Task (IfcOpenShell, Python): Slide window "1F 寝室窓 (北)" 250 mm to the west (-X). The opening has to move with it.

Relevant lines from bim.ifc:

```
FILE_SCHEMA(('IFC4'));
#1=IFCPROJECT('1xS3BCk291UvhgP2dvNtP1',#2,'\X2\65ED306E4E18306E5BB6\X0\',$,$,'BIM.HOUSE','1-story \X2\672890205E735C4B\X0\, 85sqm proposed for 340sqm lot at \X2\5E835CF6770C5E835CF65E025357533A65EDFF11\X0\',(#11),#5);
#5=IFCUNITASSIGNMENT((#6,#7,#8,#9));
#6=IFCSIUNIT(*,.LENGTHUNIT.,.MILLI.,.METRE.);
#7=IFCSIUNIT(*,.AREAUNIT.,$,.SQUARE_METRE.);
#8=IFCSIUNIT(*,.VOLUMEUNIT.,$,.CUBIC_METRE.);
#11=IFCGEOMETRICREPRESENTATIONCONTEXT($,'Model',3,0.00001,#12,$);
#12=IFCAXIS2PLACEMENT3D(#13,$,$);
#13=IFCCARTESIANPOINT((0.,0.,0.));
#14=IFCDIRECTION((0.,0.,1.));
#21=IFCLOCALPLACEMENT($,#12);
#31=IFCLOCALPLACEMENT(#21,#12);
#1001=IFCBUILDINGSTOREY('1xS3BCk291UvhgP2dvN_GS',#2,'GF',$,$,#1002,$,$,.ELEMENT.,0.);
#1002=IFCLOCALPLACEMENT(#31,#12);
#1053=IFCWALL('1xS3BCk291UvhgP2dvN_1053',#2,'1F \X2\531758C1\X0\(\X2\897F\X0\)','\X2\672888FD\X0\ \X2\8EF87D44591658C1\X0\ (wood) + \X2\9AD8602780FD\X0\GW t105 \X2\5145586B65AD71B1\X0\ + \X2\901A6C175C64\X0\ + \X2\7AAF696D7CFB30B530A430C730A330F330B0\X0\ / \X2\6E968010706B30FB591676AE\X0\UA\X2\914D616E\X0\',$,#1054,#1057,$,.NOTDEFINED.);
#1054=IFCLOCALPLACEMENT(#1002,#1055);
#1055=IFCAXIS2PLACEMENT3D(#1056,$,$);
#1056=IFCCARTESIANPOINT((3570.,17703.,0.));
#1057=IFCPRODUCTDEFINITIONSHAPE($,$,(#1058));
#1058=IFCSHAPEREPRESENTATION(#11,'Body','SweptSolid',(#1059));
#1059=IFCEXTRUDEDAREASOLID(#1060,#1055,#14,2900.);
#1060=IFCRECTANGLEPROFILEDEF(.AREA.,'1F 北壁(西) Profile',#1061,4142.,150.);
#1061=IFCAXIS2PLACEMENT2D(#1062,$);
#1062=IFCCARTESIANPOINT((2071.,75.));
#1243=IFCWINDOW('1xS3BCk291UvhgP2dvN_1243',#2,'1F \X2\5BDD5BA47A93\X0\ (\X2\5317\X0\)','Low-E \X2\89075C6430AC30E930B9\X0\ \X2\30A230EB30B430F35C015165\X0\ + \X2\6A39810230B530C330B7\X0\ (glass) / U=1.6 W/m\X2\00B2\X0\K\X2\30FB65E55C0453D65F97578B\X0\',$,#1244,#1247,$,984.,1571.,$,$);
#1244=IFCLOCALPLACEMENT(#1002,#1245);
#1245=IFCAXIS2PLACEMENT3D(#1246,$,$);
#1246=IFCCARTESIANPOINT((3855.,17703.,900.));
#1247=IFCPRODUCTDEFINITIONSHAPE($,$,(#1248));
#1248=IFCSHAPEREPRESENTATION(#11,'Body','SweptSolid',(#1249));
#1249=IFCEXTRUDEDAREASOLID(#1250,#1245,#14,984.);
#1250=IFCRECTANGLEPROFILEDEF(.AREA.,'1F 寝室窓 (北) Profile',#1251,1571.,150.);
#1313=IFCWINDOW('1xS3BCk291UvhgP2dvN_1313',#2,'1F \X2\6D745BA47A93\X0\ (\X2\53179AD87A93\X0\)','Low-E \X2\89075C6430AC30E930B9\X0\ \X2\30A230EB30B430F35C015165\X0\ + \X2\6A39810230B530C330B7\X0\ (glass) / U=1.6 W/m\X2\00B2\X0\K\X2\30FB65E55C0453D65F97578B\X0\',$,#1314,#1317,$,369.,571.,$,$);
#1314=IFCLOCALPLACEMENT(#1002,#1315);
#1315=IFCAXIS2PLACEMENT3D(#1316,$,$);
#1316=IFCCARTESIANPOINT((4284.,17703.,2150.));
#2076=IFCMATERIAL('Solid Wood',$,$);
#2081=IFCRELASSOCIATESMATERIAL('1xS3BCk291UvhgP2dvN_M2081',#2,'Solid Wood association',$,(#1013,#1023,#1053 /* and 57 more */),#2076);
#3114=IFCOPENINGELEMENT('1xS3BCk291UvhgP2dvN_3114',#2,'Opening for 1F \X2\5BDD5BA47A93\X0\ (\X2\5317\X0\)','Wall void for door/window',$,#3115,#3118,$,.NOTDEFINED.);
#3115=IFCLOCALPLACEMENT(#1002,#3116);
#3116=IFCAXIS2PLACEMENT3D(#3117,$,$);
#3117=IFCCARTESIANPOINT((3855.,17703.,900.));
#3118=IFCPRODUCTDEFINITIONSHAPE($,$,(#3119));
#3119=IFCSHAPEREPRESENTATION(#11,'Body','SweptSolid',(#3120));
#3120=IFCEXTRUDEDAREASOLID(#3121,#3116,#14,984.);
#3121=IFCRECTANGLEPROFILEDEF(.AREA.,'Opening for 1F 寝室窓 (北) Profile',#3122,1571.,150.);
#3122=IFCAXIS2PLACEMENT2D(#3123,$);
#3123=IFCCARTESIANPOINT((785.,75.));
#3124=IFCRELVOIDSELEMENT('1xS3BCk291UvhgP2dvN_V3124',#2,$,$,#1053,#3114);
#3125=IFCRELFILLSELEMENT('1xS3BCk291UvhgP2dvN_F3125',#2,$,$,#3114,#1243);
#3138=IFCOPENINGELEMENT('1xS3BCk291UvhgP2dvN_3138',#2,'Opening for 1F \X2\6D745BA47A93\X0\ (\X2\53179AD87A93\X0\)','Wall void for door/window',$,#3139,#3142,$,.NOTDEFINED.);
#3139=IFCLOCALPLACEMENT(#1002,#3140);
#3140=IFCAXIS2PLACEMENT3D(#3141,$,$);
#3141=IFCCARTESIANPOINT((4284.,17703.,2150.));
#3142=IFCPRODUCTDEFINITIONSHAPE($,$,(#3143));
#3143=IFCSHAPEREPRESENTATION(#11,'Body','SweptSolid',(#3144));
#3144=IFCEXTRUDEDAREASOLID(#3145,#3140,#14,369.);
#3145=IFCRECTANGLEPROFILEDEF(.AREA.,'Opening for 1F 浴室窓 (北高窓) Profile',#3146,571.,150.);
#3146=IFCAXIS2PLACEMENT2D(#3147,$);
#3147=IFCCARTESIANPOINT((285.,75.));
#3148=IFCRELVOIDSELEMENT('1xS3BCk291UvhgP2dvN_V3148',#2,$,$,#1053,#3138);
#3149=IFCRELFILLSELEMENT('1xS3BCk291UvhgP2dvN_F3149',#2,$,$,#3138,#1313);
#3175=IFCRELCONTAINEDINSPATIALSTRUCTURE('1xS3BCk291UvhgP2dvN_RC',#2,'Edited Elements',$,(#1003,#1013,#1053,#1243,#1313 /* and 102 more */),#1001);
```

```python
import ifcopenshell
import ifcopenshell.api.geometry
import ifcopenshell.util.placement
import ifcopenshell.util.unit

model = ifcopenshell.open("bim.ifc")
unit_scale = ifcopenshell.util.unit.calculate_unit_scale(model)

window = model.by_id(1243)
opening = window.FillsVoids[0].RelatingOpeningElement
wall = opening.VoidsElements[0].RelatingBuildingElement

wall_matrix = ifcopenshell.util.placement.get_local_placement(wall.ObjectPlacement)
shift = wall_matrix[:3, 0] * -0.25 / unit_scale
before = ifcopenshell.util.placement.get_local_placement(window.ObjectPlacement)[:3, 3].copy()

# The window is not placed relative to its opening, so move both.
for product in (opening, window):
    matrix = ifcopenshell.util.placement.get_local_placement(product.ObjectPlacement)
    matrix[:3, 3] += shift
    ifcopenshell.api.geometry.edit_object_placement(model, product=product, matrix=matrix, is_si=False)

after = ifcopenshell.util.placement.get_local_placement(window.ObjectPlacement)[:3, 3]
print("window moved by", (after - before).round(3) + 0.0)

model.write("bim_updated.ifc")
```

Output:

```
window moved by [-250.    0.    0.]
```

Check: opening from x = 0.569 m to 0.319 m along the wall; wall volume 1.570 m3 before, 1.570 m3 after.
